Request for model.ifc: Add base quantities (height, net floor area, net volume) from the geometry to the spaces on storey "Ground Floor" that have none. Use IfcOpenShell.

First a look at what the model holds.

```python
import ifcopenshell
import ifcopenshell.util.element
import ifcopenshell.util.unit

model = ifcopenshell.open("model.ifc")
print(model.schema)
for unit_type in ("LENGTHUNIT", "AREAUNIT", "VOLUMEUNIT"):
    print(unit_type, ifcopenshell.util.unit.calculate_unit_scale(model, unit_type))
storey = next(s for s in model.by_type("IfcBuildingStorey") if s.Name == "Ground Floor")
spaces = [e for e in ifcopenshell.util.element.get_decomposition(storey) if e.is_a("IfcSpace")]
for e in sorted(spaces, key=lambda e: e.id()):
    print(e.id(), e.is_a(), e.Name, list(ifcopenshell.util.element.get_psets(e, qtos_only=True)), sep=" | ")
```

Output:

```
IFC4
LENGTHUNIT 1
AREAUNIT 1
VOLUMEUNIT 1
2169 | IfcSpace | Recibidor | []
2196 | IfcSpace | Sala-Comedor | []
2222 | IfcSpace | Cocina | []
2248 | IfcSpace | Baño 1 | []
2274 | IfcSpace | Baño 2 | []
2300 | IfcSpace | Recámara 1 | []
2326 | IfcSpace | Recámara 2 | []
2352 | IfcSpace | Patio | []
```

```python
import ifcopenshell
import ifcopenshell.api.pset
import ifcopenshell.geom
import ifcopenshell.util.element
import ifcopenshell.util.shape
import ifcopenshell.util.unit

model = ifcopenshell.open("model.ifc")
unit_scale = ifcopenshell.util.unit.calculate_unit_scale(model)
area_scale = ifcopenshell.util.unit.calculate_unit_scale(model, "AREAUNIT")
volume_scale = ifcopenshell.util.unit.calculate_unit_scale(model, "VOLUMEUNIT")
settings = ifcopenshell.geom.settings()

storey = next(s for s in model.by_type("IfcBuildingStorey") if s.Name == "Ground Floor")
spaces = [e for e in ifcopenshell.util.element.get_decomposition(storey) if e.is_a("IfcSpace")]

for e in sorted(spaces, key=lambda e: e.id()):
    if ifcopenshell.util.element.get_psets(e, qtos_only=True, should_inherit=False):
        continue
    # Geometry comes back in metres, in the element's own axes.
    shape = ifcopenshell.geom.create_shape(settings, e)
    values = {
        "Height": ifcopenshell.util.shape.get_z(shape.geometry) / unit_scale,
        "NetFloorArea": ifcopenshell.util.shape.get_footprint_area(shape.geometry) / area_scale,
        "NetVolume": ifcopenshell.util.shape.get_volume(shape.geometry) / volume_scale,
    }
    qto = ifcopenshell.api.pset.add_qto(model, product=e, name="Qto_SpaceBaseQuantities")
    ifcopenshell.api.pset.edit_qto(model, qto=qto, properties=values)
    print(e.id(), {k: round(v, 3) for k, v in values.items()})

model.write("model_rev.ifc")
```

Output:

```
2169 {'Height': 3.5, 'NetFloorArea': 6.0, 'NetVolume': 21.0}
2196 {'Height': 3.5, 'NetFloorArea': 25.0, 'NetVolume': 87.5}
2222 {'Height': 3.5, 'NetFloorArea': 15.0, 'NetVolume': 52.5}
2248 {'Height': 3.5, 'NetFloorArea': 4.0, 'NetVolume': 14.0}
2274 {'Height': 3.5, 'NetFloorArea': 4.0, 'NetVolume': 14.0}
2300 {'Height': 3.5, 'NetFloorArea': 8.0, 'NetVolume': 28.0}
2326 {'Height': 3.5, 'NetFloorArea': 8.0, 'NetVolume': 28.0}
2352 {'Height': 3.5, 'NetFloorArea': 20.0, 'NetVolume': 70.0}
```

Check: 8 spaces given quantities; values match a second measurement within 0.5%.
